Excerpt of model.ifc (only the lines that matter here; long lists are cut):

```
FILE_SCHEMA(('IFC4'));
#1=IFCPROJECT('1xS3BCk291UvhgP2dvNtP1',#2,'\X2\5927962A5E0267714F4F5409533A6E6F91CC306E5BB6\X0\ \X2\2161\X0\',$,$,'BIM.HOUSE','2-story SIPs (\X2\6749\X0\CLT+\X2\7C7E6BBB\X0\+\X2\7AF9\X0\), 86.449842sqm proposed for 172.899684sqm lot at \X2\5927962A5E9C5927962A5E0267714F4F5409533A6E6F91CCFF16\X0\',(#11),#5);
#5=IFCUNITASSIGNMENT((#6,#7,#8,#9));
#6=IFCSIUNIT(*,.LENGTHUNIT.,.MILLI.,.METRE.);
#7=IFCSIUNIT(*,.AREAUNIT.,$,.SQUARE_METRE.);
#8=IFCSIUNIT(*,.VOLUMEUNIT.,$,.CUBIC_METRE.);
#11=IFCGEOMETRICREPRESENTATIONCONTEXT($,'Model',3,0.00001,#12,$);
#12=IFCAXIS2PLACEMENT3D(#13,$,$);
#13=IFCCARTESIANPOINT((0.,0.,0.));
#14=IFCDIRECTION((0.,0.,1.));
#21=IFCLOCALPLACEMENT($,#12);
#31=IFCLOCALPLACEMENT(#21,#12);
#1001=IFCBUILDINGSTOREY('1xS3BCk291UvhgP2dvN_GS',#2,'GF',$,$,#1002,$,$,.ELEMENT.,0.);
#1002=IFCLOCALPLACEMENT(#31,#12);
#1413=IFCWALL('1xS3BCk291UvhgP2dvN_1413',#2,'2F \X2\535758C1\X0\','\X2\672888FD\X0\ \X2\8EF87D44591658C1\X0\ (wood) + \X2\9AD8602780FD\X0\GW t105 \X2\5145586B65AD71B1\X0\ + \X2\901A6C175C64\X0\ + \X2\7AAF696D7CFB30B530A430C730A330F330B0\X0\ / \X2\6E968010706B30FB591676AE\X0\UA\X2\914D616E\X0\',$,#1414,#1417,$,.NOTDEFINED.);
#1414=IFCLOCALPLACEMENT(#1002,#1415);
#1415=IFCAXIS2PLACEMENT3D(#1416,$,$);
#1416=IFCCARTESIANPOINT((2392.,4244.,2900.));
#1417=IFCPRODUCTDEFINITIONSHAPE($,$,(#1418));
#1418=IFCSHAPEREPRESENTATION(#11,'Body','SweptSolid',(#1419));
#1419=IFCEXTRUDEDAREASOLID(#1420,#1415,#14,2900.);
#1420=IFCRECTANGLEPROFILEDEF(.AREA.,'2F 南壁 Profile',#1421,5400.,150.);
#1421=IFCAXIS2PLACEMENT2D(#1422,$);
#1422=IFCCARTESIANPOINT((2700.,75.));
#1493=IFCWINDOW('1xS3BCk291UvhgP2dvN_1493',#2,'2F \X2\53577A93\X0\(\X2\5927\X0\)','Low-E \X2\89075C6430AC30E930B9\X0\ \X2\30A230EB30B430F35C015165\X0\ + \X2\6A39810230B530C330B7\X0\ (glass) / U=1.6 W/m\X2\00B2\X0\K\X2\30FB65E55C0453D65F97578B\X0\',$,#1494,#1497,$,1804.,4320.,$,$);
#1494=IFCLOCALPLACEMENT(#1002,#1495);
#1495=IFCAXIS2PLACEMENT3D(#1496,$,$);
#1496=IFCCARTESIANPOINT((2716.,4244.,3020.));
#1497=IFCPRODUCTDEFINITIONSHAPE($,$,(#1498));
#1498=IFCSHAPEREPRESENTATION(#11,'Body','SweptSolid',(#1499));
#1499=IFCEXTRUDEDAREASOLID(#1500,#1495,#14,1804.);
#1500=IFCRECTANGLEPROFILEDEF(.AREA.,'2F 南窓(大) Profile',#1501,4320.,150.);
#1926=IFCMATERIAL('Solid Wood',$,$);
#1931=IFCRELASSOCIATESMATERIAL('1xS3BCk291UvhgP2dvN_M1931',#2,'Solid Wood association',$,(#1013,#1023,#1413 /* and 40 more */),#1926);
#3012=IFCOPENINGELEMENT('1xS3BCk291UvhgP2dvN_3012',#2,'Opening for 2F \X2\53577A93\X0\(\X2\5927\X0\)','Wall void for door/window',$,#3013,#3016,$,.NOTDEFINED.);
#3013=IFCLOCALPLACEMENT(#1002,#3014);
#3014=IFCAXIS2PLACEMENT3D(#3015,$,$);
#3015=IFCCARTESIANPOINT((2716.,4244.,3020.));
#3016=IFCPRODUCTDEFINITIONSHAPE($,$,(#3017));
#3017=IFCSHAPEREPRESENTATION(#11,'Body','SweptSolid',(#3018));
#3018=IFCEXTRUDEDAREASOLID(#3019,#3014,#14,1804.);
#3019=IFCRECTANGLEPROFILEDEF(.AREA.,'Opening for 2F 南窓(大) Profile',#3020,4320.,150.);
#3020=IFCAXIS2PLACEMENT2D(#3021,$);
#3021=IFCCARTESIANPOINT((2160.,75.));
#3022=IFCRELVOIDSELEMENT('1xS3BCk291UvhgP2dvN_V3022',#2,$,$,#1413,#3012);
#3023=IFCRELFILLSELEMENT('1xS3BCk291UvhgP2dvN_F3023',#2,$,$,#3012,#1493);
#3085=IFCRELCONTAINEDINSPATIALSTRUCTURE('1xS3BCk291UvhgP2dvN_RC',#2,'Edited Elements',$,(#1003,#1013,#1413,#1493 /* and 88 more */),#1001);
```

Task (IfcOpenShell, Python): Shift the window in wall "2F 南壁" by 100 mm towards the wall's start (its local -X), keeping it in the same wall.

```python
import ifcopenshell
import ifcopenshell.api.geometry
import ifcopenshell.util.placement
import ifcopenshell.util.unit

model = ifcopenshell.open("model.ifc")
unit_scale = ifcopenshell.util.unit.calculate_unit_scale(model)

window = model.by_guid("1xS3BCk291UvhgP2dvN_1493")
opening = window.FillsVoids[0].RelatingOpeningElement
wall = opening.VoidsElements[0].RelatingBuildingElement

wall_matrix = ifcopenshell.util.placement.get_local_placement(wall.ObjectPlacement)
shift = wall_matrix[:3, 0] * -0.1 / unit_scale
before = ifcopenshell.util.placement.get_local_placement(window.ObjectPlacement)[:3, 3].copy()

# The window is not placed relative to its opening, so move both.
for product in (opening, window):
    matrix = ifcopenshell.util.placement.get_local_placement(product.ObjectPlacement)
    matrix[:3, 3] += shift
    ifcopenshell.api.geometry.edit_object_placement(model, product=product, matrix=matrix, is_si=False)

after = ifcopenshell.util.placement.get_local_placement(window.ObjectPlacement)[:3, 3]
print("window moved by", (after - before).round(3) + 0.0)

model.write("model_updated.ifc")
```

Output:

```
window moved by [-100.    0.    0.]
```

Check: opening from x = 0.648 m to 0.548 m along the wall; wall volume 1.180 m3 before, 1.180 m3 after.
